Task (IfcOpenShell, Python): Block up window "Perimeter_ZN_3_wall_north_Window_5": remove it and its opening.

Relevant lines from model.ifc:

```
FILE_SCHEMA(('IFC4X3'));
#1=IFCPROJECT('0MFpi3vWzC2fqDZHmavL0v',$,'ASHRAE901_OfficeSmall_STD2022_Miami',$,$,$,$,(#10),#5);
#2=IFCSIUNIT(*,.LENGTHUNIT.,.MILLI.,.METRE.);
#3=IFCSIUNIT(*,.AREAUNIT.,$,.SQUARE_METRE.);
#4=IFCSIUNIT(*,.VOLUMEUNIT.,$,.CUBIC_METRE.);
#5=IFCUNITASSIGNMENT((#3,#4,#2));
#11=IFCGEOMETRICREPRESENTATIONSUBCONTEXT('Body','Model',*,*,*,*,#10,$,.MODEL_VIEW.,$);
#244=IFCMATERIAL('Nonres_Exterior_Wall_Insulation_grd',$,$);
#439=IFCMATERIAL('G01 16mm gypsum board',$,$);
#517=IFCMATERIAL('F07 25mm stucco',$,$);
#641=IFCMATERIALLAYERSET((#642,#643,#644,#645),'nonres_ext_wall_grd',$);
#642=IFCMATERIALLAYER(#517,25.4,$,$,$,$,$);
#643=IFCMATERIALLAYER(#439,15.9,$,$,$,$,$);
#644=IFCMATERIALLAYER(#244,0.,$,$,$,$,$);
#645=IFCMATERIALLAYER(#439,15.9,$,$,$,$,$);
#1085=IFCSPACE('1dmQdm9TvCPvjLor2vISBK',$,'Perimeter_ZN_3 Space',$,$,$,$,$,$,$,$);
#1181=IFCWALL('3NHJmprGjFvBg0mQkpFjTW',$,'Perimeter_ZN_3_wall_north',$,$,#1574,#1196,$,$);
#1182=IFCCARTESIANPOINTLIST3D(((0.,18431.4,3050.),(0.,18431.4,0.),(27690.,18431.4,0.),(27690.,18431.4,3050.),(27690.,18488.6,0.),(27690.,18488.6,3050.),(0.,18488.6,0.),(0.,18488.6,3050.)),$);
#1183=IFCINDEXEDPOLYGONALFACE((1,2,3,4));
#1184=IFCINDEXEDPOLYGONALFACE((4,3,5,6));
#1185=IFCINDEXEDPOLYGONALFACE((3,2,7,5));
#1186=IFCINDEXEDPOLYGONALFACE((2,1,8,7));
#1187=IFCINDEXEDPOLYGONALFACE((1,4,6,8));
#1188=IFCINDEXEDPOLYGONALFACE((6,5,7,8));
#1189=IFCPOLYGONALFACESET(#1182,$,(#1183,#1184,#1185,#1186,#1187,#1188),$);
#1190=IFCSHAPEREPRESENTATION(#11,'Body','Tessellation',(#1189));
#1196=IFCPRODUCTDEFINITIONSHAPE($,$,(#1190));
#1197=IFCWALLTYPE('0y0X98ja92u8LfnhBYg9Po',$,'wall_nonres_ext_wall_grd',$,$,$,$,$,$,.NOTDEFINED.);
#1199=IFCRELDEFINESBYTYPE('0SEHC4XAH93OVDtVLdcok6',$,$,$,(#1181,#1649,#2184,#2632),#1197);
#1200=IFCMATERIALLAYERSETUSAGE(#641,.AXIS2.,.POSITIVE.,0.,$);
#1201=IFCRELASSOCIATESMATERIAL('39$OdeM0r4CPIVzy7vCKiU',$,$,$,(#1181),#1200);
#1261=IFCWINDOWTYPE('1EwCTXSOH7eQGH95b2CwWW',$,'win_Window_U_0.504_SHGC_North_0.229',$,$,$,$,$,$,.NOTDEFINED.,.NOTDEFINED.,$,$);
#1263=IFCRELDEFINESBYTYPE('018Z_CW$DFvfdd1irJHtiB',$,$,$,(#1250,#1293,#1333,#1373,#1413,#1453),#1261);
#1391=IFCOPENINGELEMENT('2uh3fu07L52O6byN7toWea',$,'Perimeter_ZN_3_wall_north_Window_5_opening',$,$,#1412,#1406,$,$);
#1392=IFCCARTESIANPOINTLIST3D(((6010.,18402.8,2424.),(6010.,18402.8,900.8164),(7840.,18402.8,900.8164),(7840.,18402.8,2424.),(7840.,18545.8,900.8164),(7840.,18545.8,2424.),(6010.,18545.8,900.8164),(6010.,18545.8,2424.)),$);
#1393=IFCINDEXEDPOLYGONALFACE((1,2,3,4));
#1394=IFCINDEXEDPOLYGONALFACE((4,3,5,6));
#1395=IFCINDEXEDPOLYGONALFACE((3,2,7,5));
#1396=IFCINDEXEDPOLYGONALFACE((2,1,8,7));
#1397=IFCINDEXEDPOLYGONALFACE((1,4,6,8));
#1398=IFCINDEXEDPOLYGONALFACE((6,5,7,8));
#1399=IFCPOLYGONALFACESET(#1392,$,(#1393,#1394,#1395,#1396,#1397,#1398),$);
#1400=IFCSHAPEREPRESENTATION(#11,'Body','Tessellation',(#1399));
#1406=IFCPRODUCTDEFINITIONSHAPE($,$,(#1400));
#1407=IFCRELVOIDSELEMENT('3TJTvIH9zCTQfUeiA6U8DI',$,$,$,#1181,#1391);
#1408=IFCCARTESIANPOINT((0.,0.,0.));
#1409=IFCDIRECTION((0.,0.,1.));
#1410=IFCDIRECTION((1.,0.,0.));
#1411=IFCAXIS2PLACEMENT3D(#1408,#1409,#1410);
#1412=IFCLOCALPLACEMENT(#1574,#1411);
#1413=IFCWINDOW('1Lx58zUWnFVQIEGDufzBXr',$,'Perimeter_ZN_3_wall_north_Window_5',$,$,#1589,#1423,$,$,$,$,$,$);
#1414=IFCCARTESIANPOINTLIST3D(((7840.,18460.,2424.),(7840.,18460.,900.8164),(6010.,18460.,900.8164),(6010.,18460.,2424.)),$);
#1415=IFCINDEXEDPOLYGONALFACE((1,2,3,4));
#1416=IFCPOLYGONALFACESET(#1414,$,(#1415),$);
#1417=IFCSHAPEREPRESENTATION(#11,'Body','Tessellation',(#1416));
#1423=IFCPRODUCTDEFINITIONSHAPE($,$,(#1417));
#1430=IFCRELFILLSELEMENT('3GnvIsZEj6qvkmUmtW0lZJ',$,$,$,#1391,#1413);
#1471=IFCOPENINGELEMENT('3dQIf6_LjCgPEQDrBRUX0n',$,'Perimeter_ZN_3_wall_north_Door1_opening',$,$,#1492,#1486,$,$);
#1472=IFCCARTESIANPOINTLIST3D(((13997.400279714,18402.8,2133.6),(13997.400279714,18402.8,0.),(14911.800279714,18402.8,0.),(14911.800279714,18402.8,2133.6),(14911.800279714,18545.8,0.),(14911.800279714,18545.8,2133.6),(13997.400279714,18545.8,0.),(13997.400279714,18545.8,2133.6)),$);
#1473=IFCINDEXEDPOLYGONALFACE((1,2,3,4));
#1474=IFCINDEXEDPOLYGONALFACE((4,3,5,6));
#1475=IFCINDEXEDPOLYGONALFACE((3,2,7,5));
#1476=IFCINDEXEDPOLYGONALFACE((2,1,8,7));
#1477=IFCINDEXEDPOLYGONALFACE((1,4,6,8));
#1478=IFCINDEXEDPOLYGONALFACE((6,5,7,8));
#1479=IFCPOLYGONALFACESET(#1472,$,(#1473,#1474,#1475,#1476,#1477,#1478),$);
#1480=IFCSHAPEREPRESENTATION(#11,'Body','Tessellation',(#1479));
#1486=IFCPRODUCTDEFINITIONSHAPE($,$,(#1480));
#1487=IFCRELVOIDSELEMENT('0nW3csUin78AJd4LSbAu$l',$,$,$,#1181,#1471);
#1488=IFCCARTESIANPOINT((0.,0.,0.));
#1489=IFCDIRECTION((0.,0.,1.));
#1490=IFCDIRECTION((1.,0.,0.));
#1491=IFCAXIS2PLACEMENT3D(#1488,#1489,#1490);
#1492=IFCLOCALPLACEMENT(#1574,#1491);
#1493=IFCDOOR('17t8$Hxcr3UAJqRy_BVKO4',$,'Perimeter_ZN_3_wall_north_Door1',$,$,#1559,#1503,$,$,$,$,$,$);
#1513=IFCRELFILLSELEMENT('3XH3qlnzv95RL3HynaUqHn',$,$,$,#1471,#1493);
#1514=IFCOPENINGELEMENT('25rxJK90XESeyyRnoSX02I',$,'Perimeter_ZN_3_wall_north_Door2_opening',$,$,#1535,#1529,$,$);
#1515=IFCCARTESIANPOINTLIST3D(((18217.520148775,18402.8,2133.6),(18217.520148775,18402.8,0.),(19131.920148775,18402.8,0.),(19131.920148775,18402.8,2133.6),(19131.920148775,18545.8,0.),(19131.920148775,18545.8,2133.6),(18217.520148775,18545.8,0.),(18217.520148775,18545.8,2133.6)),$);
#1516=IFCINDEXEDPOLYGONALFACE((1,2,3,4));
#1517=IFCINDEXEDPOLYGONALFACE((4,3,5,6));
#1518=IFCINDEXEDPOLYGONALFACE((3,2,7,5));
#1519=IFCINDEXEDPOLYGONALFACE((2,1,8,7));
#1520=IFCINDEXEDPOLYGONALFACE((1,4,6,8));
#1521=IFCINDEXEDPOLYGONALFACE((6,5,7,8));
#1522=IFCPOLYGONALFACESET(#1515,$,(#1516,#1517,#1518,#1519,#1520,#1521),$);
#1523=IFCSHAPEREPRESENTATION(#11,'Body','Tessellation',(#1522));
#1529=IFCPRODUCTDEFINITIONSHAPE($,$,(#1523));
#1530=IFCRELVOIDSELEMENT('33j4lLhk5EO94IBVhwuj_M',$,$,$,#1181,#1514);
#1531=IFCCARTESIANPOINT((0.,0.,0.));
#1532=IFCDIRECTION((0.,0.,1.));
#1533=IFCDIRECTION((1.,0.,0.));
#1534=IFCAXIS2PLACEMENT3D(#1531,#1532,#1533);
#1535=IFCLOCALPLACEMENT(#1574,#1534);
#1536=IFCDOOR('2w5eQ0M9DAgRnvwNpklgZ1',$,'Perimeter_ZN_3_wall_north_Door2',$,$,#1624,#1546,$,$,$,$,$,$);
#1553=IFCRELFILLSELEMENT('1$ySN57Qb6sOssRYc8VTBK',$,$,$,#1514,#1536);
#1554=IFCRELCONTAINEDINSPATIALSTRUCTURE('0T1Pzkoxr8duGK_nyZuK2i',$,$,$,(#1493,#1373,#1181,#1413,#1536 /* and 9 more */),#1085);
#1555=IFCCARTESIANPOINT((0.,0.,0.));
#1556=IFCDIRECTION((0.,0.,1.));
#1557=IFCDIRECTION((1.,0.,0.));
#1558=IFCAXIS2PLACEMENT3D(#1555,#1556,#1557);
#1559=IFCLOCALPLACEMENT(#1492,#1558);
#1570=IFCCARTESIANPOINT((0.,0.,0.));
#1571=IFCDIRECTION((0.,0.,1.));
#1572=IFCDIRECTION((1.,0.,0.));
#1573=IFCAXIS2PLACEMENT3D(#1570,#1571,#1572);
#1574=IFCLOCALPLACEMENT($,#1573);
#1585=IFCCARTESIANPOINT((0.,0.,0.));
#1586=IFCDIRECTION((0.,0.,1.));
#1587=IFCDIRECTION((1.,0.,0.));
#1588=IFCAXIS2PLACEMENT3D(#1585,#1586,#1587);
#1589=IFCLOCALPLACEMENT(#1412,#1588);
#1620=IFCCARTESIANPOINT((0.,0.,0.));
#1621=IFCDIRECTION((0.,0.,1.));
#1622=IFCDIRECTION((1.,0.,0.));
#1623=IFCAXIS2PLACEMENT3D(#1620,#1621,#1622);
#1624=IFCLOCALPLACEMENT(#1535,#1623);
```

```python
import ifcopenshell
import ifcopenshell.api.feature
import ifcopenshell.api.root
import ifcopenshell.geom
import ifcopenshell.util.shape

model = ifcopenshell.open("model.ifc")
settings = ifcopenshell.geom.settings()


def volume(element):
    """Net volume in cubic metres, openings subtracted."""
    shape = ifcopenshell.geom.create_shape(settings, element)
    return ifcopenshell.util.shape.get_volume(shape.geometry)


window = model.by_id(1413)
opening = window.FillsVoids[0].RelatingOpeningElement
wall = opening.VoidsElements[0].RelatingBuildingElement
before = volume(wall)

ifcopenshell.api.root.remove_product(model, product=window)
ifcopenshell.api.feature.remove_feature(model, feature=opening)

after = volume(wall)

print(f"wall volume {before:.3f} -> {after:.3f} m3")

model.write("model_updated.ifc")
```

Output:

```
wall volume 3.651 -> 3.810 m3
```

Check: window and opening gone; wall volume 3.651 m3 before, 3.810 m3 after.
